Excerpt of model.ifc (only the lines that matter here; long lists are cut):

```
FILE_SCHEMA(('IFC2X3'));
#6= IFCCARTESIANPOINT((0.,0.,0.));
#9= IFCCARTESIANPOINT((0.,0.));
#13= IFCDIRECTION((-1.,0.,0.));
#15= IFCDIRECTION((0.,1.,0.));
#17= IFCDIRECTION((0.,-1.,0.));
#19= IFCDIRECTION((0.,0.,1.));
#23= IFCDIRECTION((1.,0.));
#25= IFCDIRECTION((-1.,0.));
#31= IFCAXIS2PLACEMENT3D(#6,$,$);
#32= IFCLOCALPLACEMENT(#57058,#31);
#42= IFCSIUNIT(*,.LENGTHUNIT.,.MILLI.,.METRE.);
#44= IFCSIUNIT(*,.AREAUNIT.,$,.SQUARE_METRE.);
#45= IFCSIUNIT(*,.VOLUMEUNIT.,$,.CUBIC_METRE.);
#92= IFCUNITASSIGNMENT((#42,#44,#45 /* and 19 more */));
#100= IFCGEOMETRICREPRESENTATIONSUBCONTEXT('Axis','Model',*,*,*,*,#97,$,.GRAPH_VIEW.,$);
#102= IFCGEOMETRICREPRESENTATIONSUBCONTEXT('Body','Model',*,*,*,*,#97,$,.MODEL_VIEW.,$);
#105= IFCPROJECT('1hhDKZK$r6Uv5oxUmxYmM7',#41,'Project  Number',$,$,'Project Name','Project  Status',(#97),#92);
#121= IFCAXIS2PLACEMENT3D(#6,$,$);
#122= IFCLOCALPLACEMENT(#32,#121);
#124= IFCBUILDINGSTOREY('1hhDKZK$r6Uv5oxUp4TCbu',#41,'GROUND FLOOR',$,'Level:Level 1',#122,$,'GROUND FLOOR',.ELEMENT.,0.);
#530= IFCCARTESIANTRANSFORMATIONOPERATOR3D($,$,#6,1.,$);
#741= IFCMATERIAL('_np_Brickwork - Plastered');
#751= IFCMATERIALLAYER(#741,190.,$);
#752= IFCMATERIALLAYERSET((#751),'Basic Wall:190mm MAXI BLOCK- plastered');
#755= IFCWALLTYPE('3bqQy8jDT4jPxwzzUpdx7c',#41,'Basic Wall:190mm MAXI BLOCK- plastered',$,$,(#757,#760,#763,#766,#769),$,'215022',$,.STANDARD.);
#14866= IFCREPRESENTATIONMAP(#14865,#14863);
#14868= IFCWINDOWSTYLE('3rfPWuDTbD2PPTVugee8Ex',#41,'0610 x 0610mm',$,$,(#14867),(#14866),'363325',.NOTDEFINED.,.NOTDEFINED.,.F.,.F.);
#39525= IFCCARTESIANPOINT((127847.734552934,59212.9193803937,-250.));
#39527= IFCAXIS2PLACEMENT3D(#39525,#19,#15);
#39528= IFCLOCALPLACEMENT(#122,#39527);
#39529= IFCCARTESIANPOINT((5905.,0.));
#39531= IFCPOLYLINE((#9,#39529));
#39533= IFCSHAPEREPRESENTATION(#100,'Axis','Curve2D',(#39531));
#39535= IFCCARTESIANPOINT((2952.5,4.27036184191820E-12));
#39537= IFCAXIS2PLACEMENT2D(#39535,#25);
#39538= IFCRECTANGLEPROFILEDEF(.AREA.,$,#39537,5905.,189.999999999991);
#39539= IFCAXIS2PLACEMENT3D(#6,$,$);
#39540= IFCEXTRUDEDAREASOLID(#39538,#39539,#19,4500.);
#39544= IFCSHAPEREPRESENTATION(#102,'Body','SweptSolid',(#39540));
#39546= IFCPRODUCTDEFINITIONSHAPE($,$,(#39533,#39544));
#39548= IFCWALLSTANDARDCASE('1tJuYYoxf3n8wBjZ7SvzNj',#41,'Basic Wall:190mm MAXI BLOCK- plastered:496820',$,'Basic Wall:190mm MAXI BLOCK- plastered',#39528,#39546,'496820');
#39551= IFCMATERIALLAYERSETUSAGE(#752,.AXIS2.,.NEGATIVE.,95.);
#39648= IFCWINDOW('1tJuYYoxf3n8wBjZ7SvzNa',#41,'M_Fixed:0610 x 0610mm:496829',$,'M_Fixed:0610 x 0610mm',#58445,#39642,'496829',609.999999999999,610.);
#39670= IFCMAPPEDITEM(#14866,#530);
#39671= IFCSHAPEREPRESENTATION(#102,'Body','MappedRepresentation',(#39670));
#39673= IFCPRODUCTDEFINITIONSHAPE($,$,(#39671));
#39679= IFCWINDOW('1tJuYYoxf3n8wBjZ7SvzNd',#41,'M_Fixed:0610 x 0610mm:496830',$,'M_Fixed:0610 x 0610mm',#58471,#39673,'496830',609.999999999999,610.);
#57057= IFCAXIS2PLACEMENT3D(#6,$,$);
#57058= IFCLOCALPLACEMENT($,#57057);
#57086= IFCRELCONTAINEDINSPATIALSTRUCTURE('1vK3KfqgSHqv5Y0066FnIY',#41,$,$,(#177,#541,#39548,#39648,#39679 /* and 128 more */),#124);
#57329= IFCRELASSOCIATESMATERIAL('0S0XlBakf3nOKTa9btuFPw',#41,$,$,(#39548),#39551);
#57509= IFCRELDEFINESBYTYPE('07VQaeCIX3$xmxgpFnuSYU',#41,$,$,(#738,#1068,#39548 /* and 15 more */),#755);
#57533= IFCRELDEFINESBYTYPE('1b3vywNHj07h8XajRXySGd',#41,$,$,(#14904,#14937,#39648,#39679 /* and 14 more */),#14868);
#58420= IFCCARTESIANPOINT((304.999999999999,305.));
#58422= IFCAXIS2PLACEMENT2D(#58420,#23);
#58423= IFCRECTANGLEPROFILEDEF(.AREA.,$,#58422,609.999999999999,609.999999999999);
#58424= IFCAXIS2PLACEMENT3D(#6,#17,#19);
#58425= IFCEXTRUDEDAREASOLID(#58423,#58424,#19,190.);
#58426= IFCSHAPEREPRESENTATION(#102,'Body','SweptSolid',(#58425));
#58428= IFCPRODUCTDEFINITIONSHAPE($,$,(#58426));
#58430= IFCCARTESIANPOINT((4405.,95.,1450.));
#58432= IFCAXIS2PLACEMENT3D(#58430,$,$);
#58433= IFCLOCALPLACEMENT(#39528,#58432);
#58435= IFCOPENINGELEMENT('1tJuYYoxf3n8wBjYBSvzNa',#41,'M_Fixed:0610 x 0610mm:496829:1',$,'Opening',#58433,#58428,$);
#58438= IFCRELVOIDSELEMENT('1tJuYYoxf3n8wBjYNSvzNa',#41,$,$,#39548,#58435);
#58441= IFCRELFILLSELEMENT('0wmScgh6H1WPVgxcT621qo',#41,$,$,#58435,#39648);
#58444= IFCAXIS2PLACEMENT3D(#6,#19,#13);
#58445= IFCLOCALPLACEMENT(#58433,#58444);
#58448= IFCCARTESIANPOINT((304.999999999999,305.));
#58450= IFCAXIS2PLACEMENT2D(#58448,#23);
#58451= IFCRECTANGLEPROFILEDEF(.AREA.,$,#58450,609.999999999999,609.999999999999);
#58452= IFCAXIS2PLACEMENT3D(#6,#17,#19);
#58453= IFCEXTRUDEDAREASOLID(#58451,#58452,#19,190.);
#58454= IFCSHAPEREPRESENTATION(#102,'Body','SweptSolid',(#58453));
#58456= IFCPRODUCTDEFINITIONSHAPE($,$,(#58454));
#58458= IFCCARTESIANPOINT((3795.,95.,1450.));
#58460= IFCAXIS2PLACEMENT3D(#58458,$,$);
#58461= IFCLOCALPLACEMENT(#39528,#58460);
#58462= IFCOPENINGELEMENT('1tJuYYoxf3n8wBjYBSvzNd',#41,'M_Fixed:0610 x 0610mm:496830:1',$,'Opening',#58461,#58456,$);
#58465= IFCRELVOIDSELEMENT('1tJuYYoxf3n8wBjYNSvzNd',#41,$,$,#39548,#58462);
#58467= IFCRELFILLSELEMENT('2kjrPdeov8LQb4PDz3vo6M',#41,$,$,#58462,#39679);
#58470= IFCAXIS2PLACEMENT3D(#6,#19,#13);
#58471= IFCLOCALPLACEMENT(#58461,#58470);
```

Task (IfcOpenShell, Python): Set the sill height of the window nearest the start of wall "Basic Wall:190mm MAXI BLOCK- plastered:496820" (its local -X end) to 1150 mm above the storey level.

```python
import numpy as np
import ifcopenshell
import ifcopenshell.api.geometry
import ifcopenshell.geom
import ifcopenshell.util.element
import ifcopenshell.util.placement
import ifcopenshell.util.shape
import ifcopenshell.util.unit

model = ifcopenshell.open("model.ifc")
unit_scale = ifcopenshell.util.unit.calculate_unit_scale(model)

window = model.by_guid("1tJuYYoxf3n8wBjZ7SvzNd")
opening = window.FillsVoids[0].RelatingOpeningElement
storey = ifcopenshell.util.element.get_container(window, ifc_class="IfcBuildingStorey")
level = ifcopenshell.util.placement.get_local_placement(storey.ObjectPlacement)[2, 3]

# The opening's origin need not be at the sill, so measure its lowest point.
shape = ifcopenshell.geom.create_shape(ifcopenshell.geom.settings(), opening)
bottom = ifcopenshell.util.shape.get_shape_bottom_elevation(shape, shape.geometry) / unit_scale
dz = level + 1.15 / unit_scale - bottom

shift = np.array([0.0, 0.0, dz])
# The window is placed relative to its opening, so it follows when the opening moves.
matrix = ifcopenshell.util.placement.get_local_placement(opening.ObjectPlacement)
matrix[:3, 3] += shift
ifcopenshell.api.geometry.edit_object_placement(
    model, product=opening, matrix=matrix, is_si=False, should_transform_children=True
)

print(f"moved by {dz * unit_scale:+.3f} m")

model.write("model_updated.ifc")
```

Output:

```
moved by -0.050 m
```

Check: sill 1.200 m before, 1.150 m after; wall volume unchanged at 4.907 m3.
